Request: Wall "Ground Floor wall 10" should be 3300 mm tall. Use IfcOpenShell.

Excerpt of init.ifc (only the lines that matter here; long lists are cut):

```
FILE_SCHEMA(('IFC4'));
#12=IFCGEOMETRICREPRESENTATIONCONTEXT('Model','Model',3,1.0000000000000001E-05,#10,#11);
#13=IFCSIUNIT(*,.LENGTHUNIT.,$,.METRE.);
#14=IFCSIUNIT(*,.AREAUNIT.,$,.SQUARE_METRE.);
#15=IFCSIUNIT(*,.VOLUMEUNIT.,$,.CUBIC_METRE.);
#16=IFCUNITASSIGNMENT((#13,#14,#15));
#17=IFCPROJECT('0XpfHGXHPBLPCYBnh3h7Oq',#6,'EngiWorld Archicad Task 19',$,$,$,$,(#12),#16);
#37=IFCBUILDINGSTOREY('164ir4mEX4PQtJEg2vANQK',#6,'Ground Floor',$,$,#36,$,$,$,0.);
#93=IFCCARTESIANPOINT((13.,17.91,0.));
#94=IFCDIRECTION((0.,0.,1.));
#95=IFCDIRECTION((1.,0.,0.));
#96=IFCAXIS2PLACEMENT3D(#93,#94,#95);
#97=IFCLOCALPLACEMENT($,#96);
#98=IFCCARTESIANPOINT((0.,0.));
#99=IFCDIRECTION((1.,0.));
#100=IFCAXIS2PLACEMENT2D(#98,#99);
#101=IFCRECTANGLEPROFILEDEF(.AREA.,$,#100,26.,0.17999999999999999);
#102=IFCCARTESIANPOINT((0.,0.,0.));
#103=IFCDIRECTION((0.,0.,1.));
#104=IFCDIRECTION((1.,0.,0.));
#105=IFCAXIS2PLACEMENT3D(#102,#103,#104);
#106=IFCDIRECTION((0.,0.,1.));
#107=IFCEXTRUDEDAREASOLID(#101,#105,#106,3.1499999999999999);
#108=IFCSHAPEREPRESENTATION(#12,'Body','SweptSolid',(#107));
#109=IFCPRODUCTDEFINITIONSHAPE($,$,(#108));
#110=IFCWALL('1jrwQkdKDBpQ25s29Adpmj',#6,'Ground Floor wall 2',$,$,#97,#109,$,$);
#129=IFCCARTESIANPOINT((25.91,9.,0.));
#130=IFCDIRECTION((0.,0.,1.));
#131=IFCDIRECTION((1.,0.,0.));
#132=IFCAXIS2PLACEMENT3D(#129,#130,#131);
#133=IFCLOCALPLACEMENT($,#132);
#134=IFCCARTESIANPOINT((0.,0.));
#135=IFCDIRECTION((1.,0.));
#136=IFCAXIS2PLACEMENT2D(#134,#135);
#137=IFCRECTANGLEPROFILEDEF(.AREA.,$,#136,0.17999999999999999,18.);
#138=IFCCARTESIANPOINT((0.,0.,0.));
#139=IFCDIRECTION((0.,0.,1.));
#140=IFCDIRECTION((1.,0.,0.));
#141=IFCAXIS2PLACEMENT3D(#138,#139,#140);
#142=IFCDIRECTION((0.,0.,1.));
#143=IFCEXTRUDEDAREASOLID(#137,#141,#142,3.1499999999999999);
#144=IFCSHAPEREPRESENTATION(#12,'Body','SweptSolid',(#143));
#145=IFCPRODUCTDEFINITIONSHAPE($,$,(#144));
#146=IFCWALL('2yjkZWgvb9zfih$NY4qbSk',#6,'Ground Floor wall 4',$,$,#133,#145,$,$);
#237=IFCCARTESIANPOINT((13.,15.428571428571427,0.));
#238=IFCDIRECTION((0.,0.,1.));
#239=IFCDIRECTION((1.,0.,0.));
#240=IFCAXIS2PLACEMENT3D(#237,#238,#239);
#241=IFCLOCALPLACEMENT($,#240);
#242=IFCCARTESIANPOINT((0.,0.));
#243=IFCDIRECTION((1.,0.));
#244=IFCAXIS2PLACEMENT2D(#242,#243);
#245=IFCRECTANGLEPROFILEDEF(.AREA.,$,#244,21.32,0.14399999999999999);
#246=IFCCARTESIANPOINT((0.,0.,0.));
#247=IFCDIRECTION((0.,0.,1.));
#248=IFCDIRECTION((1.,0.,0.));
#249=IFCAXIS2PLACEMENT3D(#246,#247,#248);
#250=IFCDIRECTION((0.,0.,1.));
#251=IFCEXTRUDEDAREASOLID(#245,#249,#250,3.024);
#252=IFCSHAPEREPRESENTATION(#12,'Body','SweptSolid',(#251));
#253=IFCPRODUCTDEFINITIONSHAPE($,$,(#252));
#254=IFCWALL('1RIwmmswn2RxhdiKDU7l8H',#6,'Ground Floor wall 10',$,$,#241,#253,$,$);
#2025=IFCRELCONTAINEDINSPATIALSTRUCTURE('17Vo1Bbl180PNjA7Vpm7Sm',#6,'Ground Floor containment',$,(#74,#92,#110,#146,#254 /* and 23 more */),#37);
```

```python
import ifcopenshell
import ifcopenshell.geom
import ifcopenshell.util.shape

model = ifcopenshell.open("init.ifc")
settings = ifcopenshell.geom.settings()


def volume(element):
    """Net volume in cubic metres, openings subtracted."""
    shape = ifcopenshell.geom.create_shape(settings, element)
    return ifcopenshell.util.shape.get_volume(shape.geometry)


wall = model.by_guid("1RIwmmswn2RxhdiKDU7l8H")
before = volume(wall)

body = next(r for r in wall.Representation.Representations if r.RepresentationIdentifier == "Body")
solid = body.Items[0]
old_height = solid.Depth
solid.Depth = 3.3
after = volume(wall)

print(f"height {old_height:g} -> {solid.Depth:g}, volume {before:.3f} -> {after:.3f} m3")

model.write("init_rev.ifc")
```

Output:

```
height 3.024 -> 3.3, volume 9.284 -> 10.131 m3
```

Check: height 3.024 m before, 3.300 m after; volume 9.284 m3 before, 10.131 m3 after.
